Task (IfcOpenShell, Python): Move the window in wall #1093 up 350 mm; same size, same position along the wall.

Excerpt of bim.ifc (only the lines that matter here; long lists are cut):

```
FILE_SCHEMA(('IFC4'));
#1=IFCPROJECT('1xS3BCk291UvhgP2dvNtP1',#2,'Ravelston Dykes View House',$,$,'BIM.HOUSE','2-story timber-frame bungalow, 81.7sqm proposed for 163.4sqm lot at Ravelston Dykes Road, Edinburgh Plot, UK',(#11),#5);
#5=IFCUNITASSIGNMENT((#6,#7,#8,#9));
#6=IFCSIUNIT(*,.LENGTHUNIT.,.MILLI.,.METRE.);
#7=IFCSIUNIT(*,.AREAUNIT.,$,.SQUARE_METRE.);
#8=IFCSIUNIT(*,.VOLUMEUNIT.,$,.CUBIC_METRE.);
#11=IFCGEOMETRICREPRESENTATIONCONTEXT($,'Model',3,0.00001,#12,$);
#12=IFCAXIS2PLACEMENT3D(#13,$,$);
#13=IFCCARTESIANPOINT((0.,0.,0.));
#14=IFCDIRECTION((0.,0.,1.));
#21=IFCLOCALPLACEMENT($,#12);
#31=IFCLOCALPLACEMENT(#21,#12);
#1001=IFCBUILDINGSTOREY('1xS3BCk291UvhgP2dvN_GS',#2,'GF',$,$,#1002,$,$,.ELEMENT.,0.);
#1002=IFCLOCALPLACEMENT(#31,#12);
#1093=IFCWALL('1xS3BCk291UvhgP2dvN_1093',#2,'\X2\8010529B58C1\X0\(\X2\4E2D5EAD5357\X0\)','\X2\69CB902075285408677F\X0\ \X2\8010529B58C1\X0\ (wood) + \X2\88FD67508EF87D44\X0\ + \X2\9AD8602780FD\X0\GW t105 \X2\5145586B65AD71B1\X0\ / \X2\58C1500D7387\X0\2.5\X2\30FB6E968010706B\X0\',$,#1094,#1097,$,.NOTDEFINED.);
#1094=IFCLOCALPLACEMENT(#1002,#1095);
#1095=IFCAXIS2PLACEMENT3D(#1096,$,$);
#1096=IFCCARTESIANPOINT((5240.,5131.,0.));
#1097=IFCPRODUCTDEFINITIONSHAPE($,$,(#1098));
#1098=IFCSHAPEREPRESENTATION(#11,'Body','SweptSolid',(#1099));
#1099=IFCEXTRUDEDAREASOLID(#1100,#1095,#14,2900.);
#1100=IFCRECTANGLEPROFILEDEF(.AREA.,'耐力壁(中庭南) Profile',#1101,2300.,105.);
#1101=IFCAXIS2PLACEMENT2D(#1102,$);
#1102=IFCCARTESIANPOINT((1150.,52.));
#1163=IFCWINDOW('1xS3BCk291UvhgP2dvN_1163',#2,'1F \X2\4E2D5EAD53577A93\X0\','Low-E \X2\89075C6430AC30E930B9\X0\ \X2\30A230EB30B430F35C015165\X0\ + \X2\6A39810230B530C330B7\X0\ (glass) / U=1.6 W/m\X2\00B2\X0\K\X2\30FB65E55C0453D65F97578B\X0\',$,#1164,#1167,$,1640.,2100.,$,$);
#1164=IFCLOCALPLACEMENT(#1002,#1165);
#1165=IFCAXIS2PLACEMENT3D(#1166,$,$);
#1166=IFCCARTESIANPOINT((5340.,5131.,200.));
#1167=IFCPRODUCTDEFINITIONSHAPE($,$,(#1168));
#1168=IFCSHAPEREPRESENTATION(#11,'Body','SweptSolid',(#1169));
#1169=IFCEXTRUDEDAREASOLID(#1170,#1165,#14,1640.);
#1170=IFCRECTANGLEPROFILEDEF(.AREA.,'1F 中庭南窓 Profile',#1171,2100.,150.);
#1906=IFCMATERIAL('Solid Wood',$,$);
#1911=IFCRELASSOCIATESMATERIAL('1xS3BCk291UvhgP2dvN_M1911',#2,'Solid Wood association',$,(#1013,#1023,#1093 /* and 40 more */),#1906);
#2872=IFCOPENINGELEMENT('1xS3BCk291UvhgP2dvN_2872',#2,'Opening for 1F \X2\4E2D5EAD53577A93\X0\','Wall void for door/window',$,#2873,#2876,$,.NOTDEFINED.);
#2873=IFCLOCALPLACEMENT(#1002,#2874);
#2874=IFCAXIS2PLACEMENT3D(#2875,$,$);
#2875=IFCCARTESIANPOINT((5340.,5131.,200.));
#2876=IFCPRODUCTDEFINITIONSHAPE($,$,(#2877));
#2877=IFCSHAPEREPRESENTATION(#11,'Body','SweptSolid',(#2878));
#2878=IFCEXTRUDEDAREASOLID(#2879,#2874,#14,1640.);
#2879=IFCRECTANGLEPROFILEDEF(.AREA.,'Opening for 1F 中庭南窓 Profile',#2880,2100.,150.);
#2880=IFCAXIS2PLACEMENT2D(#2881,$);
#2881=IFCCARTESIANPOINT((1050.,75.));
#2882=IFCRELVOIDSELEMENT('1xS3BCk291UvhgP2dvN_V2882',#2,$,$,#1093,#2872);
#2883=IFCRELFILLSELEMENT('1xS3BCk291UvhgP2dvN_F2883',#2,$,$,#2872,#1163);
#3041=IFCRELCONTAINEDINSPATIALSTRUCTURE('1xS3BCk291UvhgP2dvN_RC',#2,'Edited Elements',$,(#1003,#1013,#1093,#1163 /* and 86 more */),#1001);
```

```python
import numpy as np
import ifcopenshell
import ifcopenshell.api.geometry
import ifcopenshell.util.placement
import ifcopenshell.util.unit

model = ifcopenshell.open("bim.ifc")
unit_scale = ifcopenshell.util.unit.calculate_unit_scale(model)

window = model.by_guid("1xS3BCk291UvhgP2dvN_1163")
opening = window.FillsVoids[0].RelatingOpeningElement
dz = 0.35 / unit_scale

shift = np.array([0.0, 0.0, dz])
# The window is not placed relative to its opening, so move both.
for product in (opening, window):
    matrix = ifcopenshell.util.placement.get_local_placement(product.ObjectPlacement)
    matrix[:3, 3] += shift
    ifcopenshell.api.geometry.edit_object_placement(model, product=product, matrix=matrix, is_si=False)

print(f"moved by {dz * unit_scale:+.3f} m")

model.write("bim_rev.ifc")
```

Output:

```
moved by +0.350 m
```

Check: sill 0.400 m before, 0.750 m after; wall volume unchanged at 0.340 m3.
